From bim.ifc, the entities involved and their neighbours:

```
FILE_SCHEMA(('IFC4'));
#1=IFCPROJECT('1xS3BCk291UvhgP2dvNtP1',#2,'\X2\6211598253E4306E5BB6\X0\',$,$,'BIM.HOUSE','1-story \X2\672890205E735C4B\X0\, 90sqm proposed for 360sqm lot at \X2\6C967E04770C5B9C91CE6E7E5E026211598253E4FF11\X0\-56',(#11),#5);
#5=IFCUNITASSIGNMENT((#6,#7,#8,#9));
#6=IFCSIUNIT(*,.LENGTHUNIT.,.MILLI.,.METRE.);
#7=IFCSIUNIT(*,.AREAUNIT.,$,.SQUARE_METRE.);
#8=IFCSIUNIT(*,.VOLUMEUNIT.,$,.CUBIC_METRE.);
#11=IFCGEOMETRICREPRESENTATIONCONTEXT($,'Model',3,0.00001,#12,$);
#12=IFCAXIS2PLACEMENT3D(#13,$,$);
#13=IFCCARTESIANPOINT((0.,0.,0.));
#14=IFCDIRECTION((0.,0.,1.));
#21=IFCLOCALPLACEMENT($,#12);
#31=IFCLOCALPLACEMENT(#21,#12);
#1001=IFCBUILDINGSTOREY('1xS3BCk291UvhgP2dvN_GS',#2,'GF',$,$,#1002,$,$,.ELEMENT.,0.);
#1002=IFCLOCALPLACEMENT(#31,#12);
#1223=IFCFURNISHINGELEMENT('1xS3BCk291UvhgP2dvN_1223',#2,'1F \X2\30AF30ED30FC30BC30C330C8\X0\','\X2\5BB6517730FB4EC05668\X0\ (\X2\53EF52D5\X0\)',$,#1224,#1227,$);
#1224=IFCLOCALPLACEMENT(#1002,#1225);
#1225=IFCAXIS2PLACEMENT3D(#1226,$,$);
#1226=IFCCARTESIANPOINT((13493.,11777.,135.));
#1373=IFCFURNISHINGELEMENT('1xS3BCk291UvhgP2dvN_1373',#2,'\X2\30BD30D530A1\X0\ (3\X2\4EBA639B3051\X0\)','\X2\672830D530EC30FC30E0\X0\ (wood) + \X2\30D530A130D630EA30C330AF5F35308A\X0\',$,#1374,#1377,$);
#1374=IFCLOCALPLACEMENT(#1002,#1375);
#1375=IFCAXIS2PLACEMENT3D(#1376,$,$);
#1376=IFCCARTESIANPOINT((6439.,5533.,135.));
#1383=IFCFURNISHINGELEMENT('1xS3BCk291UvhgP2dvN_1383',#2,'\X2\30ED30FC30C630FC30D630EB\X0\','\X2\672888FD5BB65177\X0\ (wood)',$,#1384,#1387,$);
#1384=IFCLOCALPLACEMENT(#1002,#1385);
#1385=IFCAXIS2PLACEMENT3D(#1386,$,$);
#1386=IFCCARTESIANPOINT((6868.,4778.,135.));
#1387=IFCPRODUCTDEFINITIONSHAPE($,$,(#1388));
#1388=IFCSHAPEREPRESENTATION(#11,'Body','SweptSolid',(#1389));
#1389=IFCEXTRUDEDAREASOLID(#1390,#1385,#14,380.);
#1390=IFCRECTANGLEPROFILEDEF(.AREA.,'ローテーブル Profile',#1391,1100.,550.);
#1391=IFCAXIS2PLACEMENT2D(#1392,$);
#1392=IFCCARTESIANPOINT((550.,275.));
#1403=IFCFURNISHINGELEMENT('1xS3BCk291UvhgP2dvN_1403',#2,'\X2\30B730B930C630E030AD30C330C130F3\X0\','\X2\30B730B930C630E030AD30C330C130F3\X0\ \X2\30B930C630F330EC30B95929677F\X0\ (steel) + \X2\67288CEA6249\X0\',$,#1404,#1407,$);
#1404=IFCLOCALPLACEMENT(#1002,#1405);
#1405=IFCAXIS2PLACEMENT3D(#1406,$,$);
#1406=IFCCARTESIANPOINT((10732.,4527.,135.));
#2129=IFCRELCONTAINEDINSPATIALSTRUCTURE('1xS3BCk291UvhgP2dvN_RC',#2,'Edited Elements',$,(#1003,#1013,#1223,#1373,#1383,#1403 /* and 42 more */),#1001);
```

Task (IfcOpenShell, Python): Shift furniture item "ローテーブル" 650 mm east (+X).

```python
import ifcopenshell
import ifcopenshell.api.geometry
import ifcopenshell.util.placement
import ifcopenshell.util.unit

model = ifcopenshell.open("bim.ifc")
unit_scale = ifcopenshell.util.unit.calculate_unit_scale(model)

item = model.by_id(1383)
matrix = ifcopenshell.util.placement.get_local_placement(item.ObjectPlacement)
matrix[0, 3] += 0.65 / unit_scale
ifcopenshell.api.geometry.edit_object_placement(model, product=item, matrix=matrix, is_si=False)

print(ifcopenshell.util.placement.get_local_placement(item.ObjectPlacement).round(3) + 0.0)

model.write("bim_rev.ifc")
```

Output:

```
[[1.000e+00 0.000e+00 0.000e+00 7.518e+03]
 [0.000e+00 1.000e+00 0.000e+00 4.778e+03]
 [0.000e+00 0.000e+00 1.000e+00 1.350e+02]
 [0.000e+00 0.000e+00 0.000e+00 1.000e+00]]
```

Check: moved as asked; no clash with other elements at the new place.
